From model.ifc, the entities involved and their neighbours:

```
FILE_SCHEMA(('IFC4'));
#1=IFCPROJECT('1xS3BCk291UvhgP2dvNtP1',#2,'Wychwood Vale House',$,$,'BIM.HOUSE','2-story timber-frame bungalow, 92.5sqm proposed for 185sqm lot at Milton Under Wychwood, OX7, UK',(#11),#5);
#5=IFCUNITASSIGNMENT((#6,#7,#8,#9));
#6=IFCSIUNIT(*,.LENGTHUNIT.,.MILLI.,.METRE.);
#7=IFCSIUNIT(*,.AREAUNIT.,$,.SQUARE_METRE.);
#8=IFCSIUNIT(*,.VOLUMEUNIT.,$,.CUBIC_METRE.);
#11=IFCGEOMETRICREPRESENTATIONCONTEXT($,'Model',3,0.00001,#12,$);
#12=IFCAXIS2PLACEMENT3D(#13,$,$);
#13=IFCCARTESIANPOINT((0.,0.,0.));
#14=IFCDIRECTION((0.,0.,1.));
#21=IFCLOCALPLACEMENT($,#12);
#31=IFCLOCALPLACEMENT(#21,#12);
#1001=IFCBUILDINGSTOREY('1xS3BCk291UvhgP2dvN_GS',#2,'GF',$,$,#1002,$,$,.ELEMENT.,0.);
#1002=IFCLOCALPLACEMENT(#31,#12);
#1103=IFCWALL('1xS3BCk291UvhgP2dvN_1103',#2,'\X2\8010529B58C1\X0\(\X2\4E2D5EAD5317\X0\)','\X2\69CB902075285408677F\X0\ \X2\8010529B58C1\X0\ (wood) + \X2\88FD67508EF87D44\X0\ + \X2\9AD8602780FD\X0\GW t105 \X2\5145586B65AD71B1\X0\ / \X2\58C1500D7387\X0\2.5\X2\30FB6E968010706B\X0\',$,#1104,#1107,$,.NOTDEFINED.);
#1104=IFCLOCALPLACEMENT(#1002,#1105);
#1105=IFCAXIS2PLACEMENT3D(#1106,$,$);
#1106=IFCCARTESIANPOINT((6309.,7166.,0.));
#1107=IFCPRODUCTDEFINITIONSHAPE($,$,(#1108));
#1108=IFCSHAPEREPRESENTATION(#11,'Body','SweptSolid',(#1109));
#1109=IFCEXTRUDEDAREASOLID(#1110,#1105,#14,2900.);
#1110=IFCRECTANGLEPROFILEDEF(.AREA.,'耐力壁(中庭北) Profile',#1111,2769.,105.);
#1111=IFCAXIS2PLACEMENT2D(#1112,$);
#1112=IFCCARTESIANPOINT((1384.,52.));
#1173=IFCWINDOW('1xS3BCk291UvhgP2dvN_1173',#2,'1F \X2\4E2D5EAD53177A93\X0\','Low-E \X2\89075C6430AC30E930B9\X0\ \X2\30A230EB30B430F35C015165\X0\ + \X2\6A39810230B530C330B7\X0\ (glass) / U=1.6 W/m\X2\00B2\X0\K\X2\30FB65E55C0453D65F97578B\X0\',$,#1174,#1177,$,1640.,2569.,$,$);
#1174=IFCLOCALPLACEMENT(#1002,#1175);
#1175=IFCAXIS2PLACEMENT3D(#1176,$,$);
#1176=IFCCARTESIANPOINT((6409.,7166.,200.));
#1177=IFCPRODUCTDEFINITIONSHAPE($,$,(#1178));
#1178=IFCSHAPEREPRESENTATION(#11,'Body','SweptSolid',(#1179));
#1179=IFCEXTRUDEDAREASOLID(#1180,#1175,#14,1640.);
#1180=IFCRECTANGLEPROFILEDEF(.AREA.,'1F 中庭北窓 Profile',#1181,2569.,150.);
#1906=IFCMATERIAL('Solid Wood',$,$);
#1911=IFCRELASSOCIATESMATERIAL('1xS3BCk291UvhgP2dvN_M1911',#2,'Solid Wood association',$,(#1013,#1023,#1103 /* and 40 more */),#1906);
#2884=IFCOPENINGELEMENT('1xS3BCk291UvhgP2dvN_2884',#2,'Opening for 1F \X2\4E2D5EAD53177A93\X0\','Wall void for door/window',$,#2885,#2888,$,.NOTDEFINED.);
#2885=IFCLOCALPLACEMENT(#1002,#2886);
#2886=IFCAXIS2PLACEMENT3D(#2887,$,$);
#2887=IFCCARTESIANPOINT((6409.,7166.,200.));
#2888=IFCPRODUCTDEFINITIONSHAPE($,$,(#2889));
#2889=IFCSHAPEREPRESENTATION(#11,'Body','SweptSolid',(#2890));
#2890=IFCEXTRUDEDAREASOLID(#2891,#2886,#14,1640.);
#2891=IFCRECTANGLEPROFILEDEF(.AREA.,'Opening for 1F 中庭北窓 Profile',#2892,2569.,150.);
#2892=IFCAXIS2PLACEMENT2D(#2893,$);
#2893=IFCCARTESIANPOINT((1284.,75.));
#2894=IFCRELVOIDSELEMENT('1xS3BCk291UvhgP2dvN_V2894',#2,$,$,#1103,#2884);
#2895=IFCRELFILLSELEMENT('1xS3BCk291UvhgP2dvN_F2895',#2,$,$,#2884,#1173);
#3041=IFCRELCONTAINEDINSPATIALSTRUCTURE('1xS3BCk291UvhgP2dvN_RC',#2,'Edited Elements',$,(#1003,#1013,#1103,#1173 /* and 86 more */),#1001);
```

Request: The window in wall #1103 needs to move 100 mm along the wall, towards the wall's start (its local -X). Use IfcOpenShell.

```python
import ifcopenshell
import ifcopenshell.api.geometry
import ifcopenshell.util.placement

model = ifcopenshell.open("model.ifc")

window = model.by_guid("1xS3BCk291UvhgP2dvN_1173")
opening = window.FillsVoids[0].RelatingOpeningElement
wall = opening.VoidsElements[0].RelatingBuildingElement

wall_matrix = ifcopenshell.util.placement.get_local_placement(wall.ObjectPlacement)
shift = wall_matrix[:3, 0] * -100.0
before = ifcopenshell.util.placement.get_local_placement(window.ObjectPlacement)[:3, 3].copy()

# The window is not placed relative to its opening, so move both.
for product in (opening, window):
    matrix = ifcopenshell.util.placement.get_local_placement(product.ObjectPlacement)
    matrix[:3, 3] += shift
    ifcopenshell.api.geometry.edit_object_placement(model, product=product, matrix=matrix, is_si=False)

after = ifcopenshell.util.placement.get_local_placement(window.ObjectPlacement)[:3, 3]
print("window moved by", (after - before).round(3) + 0.0)

model.write("model-out.ifc")
```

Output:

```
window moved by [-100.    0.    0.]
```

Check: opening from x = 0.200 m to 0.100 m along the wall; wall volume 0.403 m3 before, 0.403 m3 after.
